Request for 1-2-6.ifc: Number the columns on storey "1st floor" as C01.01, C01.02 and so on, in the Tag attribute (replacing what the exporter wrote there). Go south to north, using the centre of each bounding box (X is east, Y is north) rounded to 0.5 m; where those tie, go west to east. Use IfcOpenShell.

First a look at what the model holds.

```python
import ifcopenshell
import ifcopenshell.util.element
import ifcopenshell.util.placement

model = ifcopenshell.open("1-2-6.ifc")
print(model.schema)
storey = next(s for s in model.by_type("IfcBuildingStorey") if s.Name == "1st floor")
columns = [e for e in ifcopenshell.util.element.get_decomposition(storey) if e.is_a("IfcColumn")]
for e in sorted(columns, key=lambda e: e.id()):
    origin = ifcopenshell.util.placement.get_local_placement(e.ObjectPlacement)[:3, 3]
    print(e.id(), e.Tag, e.Name, origin.round(2) + 0.0, sep=" | ")
```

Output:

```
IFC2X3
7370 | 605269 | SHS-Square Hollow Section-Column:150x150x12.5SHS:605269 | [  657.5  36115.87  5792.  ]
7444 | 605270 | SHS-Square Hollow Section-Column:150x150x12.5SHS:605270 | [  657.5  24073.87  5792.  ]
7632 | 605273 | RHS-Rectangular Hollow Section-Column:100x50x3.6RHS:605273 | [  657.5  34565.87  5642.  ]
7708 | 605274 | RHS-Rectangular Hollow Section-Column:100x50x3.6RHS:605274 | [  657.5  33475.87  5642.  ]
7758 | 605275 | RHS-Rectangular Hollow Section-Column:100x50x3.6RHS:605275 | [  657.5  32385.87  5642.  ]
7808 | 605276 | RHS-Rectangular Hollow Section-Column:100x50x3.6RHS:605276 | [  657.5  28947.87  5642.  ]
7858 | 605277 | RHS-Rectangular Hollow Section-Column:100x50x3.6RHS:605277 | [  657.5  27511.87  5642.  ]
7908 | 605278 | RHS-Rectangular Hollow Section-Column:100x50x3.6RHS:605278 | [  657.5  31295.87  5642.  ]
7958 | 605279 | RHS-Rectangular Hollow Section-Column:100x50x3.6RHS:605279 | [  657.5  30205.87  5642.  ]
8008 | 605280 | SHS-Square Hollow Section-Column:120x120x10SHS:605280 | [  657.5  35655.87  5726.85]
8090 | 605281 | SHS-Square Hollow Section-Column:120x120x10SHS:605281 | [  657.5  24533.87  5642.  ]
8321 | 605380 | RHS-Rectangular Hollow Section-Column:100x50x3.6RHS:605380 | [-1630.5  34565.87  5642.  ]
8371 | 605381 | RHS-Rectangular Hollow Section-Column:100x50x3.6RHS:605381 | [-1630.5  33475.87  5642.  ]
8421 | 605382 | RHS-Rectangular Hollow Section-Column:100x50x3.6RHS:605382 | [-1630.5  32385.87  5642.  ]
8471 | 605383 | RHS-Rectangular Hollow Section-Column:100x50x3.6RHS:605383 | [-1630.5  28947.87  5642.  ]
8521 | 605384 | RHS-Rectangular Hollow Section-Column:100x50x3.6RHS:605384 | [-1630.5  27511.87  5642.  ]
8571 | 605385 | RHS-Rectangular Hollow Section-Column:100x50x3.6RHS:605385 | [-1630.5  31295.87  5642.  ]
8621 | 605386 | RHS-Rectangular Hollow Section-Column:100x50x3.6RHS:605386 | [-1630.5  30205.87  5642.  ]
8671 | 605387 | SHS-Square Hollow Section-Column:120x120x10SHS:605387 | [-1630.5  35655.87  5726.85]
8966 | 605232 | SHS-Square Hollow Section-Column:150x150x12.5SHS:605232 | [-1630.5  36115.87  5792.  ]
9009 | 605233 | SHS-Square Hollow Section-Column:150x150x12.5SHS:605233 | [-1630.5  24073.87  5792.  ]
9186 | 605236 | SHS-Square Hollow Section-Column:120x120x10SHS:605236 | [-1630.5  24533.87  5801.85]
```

```python
import ifcopenshell
import ifcopenshell.geom
import ifcopenshell.util.element
import ifcopenshell.util.shape

model = ifcopenshell.open("1-2-6.ifc")
settings = ifcopenshell.geom.settings()
settings.set("use-world-coords", True)


def centre(element):
    shape = ifcopenshell.geom.create_shape(settings, element)
    return ifcopenshell.util.shape.get_bbox_centroid(shape.geometry)


storey = next(s for s in model.by_type("IfcBuildingStorey") if s.Name == "1st floor")
columns = [e for e in ifcopenshell.util.element.get_decomposition(storey) if e.is_a("IfcColumn")]

# Insertion points can sit at a corner or the storey origin, so sort by the geometry (in metres).
centres = {e: centre(e) for e in columns}
columns.sort(key=lambda e: (round(centres[e][1] / 0.5), centres[e][0]))

for i, e in enumerate(columns, start=1):
    number = f"C01.{i:02d}"
    e.Tag = number
    print(e.id(), number)

model.write("1-2-6_edited.ifc")
```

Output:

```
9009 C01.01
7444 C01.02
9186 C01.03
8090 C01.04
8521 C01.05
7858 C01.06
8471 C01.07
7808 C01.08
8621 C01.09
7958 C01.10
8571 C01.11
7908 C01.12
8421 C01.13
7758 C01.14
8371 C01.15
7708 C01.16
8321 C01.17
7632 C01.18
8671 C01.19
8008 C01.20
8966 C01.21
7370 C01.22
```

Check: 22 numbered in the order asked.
